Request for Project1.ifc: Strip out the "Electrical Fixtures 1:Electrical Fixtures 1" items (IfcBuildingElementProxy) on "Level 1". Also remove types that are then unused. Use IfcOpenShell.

First a look at what the model holds.

```python
import ifcopenshell
import ifcopenshell.util.element

model = ifcopenshell.open("Project1.ifc")
print(model.schema)
storey = next(s for s in model.by_type("IfcBuildingStorey") if s.Name == "Level 1")
proxies = [e for e in ifcopenshell.util.element.get_decomposition(storey) if e.is_a("IfcBuildingElementProxy")]
seen = {}
for e in proxies:
    element_type = ifcopenshell.util.element.get_type(e)
    name = element_type.Name if element_type not in (None, e) else None
    seen[name] = seen.get(name, 0) + 1
for name, count in sorted(seen.items(), key=str):
    print(count, "x", name)
```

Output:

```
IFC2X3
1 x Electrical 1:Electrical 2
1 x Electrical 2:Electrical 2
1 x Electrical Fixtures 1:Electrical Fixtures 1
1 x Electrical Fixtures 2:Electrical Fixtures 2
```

```python
import ifcopenshell
import ifcopenshell.api.root
import ifcopenshell.util.element

model = ifcopenshell.open("Project1.ifc")

storey = next(s for s in model.by_type("IfcBuildingStorey") if s.Name == "Level 1")
proxies = [e for e in ifcopenshell.util.element.get_decomposition(storey) if e.is_a("IfcBuildingElementProxy")]
targets = [e for e in proxies if (t := ifcopenshell.util.element.get_type(e)) not in (None, e) and t.Name == "Electrical Fixtures 1:Electrical Fixtures 1"]
types = {ifcopenshell.util.element.get_type(e) for e in targets} - {None, *targets}

for e in targets:
    ifcopenshell.api.root.remove_product(model, product=e)
print(len(targets), "removed")

unused = [t for t in types if not ifcopenshell.util.element.get_types(t)]
for t in unused:
    ifcopenshell.api.root.remove_product(model, product=t)
print(len(unused), "unused types removed")

model.write("Project1-out.ifc")
```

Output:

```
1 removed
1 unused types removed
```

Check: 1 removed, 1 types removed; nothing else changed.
